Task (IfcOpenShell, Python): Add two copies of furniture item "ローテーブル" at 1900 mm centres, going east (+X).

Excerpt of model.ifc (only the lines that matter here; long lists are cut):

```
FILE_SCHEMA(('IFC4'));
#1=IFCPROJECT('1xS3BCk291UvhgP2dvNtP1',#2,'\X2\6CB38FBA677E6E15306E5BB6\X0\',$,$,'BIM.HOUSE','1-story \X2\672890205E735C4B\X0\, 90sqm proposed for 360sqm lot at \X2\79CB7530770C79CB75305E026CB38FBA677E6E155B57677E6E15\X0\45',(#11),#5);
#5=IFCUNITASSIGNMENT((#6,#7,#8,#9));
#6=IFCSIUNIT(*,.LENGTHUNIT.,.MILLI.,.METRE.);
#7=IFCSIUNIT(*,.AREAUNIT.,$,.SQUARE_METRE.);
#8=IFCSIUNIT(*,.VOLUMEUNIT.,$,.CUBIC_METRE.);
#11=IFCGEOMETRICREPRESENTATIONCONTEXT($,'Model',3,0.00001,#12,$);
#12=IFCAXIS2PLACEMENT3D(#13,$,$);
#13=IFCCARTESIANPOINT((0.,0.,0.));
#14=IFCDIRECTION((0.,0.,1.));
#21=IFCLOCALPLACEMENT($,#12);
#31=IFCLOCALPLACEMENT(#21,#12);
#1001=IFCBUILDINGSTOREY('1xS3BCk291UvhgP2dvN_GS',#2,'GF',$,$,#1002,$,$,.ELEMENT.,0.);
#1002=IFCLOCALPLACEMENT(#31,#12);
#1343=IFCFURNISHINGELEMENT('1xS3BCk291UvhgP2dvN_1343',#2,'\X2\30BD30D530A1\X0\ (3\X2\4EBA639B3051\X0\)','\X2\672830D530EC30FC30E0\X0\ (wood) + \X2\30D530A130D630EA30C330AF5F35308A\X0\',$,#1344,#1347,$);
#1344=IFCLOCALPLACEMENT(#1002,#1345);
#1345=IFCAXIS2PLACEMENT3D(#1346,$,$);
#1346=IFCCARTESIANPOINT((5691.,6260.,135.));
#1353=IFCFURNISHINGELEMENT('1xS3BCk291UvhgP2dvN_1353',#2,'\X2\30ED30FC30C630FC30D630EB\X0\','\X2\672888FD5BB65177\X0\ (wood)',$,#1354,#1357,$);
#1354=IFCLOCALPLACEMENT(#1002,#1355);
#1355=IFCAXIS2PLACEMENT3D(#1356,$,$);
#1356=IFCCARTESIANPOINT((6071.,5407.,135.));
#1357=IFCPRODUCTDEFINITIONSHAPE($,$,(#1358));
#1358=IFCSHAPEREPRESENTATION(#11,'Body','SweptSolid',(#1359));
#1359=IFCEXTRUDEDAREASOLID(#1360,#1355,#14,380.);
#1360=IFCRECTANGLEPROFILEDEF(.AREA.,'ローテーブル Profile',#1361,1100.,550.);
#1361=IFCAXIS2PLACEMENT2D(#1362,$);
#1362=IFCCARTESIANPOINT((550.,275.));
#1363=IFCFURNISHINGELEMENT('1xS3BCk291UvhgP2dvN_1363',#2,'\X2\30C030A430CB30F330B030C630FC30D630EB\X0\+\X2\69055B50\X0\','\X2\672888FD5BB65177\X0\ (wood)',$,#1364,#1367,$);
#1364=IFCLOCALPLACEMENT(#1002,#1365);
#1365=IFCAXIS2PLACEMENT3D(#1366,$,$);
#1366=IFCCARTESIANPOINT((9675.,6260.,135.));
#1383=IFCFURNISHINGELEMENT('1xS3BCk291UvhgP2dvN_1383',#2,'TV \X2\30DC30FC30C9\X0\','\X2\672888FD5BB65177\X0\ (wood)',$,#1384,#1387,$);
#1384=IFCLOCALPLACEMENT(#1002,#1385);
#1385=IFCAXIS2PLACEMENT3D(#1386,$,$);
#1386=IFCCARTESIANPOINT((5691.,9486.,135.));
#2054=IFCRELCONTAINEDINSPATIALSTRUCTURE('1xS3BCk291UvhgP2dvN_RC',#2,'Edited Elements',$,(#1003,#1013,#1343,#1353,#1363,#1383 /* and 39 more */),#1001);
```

```python
import numpy as np
import ifcopenshell
import ifcopenshell.api.geometry
import ifcopenshell.api.root
import ifcopenshell.util.element
import ifcopenshell.util.placement
import ifcopenshell.util.unit

model = ifcopenshell.open("model.ifc")
unit_scale = ifcopenshell.util.unit.calculate_unit_scale(model)


def reuse_history(source, copy):
    """copy_class also copies each property set's owner history, people and application; keep the originals."""
    for rel in copy.IsDefinedBy:
        if rel.is_a("IfcRelDefinesByProperties") and (history := rel.RelatingPropertyDefinition.OwnerHistory):
            rel.RelatingPropertyDefinition.OwnerHistory = source.OwnerHistory
            ifcopenshell.util.element.remove_deep2(model, history)


source = model.by_guid("1xS3BCk291UvhgP2dvN_1353")
base = ifcopenshell.util.placement.get_local_placement(source.ObjectPlacement)
step = np.array([1.0, 0.0, 0.0]) * 1.9 / unit_scale

for i in range(1, 3):
    copy = ifcopenshell.api.root.copy_class(model, product=source)
    copy.Representation = ifcopenshell.util.element.copy_deep(
        model, source.Representation, exclude=["IfcGeometricRepresentationContext", "IfcRepresentationMap"]
    )
    reuse_history(source, copy)
    matrix = base.copy()
    matrix[:3, 3] += i * step
    print("added at", matrix[:3, 3].round(3) + 0.0)
    ifcopenshell.api.geometry.edit_object_placement(model, product=copy, matrix=matrix, is_si=False)

model.write("model_rev.ifc")
```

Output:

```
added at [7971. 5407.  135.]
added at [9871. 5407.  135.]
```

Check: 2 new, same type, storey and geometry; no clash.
